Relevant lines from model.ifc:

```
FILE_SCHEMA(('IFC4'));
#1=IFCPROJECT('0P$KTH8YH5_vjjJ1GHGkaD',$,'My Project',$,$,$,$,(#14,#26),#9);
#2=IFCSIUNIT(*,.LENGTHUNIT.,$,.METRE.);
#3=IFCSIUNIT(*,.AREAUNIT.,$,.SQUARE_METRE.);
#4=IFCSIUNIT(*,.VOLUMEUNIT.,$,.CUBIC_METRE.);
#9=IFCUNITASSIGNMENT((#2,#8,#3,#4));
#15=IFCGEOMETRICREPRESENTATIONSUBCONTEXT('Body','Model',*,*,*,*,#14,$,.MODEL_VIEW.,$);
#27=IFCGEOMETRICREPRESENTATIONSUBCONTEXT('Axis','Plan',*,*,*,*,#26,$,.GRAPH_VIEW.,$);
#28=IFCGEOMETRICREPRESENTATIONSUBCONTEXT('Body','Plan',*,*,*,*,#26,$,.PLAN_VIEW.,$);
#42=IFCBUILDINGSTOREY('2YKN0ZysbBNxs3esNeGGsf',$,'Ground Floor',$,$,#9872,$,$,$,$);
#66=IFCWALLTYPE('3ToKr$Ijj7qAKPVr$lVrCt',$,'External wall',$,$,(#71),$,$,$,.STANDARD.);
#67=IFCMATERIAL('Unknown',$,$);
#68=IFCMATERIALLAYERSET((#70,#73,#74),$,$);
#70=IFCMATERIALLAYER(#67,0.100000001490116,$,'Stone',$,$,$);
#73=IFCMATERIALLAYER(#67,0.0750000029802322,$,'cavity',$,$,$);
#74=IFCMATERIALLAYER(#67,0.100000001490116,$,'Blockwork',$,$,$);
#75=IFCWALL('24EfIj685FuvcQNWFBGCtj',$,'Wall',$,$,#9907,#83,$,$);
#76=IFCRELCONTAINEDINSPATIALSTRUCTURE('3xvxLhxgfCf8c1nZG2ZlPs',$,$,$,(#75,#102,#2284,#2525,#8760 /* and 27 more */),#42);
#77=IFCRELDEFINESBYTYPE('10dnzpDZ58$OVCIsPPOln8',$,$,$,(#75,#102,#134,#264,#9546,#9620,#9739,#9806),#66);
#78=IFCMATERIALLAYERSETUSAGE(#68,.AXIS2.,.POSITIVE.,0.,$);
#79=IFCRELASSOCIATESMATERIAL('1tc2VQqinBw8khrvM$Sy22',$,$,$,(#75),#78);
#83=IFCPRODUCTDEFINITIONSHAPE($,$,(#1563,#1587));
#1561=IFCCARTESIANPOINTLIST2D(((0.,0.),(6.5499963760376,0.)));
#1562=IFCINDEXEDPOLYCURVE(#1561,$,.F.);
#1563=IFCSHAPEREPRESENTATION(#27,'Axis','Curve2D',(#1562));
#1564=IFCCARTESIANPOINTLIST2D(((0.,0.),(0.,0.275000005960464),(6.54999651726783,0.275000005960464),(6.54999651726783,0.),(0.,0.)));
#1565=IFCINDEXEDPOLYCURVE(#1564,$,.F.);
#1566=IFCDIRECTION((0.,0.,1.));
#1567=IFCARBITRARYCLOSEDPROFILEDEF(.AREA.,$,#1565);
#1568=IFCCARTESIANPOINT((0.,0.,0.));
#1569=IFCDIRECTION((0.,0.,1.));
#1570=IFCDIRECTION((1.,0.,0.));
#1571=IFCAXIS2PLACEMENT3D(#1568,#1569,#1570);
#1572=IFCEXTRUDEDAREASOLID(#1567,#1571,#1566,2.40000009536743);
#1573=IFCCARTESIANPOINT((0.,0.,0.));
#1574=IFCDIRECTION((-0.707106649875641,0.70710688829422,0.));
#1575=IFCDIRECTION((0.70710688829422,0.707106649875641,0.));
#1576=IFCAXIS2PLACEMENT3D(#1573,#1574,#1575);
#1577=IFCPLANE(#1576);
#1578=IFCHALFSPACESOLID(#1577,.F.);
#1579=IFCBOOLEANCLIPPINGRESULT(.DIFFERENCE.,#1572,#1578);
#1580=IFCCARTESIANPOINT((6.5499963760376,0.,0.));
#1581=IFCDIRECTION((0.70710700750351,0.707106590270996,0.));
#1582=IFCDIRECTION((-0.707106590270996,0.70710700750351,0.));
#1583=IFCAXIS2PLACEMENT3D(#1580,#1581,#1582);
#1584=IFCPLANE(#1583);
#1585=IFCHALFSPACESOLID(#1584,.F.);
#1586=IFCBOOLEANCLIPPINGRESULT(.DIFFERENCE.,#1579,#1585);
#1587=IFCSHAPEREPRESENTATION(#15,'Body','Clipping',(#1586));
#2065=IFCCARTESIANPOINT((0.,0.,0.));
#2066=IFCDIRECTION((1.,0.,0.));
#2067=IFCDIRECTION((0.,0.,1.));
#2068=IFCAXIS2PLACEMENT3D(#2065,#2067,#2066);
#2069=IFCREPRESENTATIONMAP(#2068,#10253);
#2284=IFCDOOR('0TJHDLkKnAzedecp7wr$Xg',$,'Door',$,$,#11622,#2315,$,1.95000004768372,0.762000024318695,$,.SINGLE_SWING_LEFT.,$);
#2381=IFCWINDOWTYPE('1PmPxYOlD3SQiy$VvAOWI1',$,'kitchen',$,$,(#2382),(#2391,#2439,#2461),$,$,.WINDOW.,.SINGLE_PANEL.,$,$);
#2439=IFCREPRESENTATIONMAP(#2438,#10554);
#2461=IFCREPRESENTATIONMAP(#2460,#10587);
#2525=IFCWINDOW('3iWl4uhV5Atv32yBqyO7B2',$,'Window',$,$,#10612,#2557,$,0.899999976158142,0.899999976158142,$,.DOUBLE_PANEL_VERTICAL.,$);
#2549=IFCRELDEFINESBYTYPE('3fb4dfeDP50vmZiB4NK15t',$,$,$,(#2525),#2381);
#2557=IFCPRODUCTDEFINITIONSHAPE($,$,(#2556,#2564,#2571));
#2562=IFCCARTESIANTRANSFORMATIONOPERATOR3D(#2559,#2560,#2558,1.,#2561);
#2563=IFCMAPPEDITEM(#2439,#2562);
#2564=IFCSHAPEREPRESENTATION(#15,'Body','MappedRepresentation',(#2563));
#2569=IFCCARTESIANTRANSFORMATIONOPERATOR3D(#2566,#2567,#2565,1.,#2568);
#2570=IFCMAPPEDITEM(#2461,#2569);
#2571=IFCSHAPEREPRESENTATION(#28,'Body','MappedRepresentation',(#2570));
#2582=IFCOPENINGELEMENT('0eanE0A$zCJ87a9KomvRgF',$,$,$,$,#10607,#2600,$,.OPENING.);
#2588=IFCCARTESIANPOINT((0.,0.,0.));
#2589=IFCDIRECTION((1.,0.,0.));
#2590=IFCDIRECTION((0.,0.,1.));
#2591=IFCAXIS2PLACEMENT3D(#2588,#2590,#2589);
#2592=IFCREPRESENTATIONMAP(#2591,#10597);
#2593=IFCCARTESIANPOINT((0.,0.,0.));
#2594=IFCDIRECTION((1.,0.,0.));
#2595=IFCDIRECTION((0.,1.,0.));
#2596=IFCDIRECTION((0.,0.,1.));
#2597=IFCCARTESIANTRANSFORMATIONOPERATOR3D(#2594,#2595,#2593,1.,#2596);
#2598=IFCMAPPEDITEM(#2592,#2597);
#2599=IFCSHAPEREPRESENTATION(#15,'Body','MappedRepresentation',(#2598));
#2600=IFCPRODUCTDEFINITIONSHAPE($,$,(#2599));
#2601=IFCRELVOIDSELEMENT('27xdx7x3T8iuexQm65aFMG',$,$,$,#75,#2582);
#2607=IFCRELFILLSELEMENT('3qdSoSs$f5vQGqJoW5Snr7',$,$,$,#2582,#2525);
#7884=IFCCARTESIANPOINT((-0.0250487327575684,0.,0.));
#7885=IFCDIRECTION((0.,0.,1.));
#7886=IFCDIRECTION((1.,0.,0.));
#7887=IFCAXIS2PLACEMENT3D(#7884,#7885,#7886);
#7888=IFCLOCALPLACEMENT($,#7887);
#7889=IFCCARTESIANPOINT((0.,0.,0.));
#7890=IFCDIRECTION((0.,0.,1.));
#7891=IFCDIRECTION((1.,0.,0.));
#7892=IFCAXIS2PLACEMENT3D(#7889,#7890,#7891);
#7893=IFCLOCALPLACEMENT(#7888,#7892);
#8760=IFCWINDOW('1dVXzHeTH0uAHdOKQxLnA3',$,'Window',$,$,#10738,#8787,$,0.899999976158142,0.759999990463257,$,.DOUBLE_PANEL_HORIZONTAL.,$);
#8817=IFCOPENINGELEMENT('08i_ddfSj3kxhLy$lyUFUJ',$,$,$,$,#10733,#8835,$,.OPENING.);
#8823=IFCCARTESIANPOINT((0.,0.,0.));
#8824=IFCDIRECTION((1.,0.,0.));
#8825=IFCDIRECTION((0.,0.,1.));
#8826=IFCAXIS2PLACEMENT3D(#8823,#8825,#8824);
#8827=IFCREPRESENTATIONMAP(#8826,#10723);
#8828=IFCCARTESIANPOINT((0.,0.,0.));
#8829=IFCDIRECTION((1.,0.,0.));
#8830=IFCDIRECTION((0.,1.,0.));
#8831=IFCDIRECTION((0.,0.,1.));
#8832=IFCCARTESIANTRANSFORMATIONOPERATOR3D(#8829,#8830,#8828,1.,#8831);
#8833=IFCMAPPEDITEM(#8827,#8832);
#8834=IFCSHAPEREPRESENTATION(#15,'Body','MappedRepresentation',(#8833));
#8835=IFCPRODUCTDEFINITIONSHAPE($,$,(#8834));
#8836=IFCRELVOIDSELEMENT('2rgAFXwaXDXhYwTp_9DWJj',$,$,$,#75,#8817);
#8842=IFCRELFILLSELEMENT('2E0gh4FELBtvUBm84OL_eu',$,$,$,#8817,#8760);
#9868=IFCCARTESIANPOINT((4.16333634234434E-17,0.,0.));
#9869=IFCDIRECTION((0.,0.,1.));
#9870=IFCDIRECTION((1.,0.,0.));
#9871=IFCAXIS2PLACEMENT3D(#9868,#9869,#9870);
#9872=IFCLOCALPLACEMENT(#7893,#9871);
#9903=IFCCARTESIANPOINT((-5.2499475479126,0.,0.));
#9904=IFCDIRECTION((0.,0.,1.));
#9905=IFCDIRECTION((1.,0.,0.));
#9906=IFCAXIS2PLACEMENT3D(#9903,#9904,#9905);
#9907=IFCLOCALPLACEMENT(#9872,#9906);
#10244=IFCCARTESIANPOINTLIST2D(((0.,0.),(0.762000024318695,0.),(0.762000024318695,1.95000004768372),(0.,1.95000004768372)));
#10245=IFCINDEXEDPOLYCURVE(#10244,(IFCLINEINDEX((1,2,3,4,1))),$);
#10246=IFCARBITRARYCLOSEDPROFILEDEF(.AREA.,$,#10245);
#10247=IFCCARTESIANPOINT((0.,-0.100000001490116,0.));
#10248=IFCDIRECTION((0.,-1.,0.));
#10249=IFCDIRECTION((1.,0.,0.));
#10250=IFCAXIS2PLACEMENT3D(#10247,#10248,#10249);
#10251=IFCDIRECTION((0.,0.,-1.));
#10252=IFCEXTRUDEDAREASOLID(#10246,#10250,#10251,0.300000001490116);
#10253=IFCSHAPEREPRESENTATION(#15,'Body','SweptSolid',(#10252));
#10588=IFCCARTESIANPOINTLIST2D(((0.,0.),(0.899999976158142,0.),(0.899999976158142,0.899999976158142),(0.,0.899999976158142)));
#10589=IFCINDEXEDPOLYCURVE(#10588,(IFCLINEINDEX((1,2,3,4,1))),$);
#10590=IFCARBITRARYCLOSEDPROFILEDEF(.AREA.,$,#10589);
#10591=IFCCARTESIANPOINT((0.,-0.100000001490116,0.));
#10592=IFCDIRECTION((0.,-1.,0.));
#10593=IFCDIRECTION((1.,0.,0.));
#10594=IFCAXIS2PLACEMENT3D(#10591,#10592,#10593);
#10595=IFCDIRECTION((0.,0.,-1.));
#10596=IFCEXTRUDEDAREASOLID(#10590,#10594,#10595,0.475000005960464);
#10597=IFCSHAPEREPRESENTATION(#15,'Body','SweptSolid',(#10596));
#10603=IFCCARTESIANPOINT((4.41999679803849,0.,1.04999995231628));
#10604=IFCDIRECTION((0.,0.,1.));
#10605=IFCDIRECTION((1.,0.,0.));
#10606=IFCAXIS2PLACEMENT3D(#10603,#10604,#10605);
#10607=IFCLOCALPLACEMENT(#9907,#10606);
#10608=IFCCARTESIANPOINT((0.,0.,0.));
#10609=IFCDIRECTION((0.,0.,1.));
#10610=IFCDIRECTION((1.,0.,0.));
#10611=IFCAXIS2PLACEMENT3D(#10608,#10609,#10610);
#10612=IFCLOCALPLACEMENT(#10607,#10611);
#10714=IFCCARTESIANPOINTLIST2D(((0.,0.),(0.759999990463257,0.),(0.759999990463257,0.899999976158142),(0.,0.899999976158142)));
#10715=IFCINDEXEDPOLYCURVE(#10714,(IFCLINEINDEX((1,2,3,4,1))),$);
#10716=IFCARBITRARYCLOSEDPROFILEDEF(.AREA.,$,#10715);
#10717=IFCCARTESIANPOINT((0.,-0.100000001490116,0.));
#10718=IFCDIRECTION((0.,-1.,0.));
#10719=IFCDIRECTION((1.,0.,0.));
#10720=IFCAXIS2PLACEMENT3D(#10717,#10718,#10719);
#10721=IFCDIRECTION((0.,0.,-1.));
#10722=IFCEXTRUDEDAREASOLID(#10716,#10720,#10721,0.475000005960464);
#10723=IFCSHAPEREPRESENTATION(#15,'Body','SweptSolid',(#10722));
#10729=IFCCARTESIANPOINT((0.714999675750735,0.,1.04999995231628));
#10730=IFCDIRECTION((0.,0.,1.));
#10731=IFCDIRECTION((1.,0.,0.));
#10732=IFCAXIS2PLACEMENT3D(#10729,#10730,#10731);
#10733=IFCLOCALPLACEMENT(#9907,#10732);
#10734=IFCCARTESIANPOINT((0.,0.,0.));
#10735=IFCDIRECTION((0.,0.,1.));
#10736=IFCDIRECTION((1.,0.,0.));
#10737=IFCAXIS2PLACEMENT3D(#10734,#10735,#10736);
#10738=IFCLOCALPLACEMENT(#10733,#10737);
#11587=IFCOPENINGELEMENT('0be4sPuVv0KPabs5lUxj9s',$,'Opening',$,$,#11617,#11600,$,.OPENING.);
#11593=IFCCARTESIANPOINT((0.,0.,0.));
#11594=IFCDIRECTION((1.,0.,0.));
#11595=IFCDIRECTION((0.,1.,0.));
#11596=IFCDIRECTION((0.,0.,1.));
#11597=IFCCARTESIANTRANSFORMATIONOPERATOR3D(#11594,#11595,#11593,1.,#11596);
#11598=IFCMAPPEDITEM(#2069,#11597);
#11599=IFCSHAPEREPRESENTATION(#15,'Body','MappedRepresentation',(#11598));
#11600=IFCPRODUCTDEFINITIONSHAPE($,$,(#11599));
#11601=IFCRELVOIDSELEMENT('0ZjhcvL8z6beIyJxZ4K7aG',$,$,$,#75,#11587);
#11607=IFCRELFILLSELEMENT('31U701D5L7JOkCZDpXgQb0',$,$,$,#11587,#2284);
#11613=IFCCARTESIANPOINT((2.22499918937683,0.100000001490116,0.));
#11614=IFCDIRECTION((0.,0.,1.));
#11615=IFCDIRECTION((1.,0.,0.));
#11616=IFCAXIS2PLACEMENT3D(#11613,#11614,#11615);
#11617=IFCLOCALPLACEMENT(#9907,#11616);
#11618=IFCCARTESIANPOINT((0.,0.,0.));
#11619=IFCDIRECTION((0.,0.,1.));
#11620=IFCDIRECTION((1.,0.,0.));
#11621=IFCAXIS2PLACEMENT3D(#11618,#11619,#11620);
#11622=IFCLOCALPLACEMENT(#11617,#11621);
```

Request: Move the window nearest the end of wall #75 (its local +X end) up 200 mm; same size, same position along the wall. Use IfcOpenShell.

```python
import numpy as np
import ifcopenshell
import ifcopenshell.api.geometry
import ifcopenshell.util.placement
import ifcopenshell.util.unit

model = ifcopenshell.open("model.ifc")
unit_scale = ifcopenshell.util.unit.calculate_unit_scale(model)

window = model.by_guid("3iWl4uhV5Atv32yBqyO7B2")
opening = window.FillsVoids[0].RelatingOpeningElement
dz = 0.2 / unit_scale

shift = np.array([0.0, 0.0, dz])
# The window is placed relative to its opening, so it follows when the opening moves.
matrix = ifcopenshell.util.placement.get_local_placement(opening.ObjectPlacement)
matrix[:3, 3] += shift
ifcopenshell.api.geometry.edit_object_placement(
    model, product=opening, matrix=matrix, is_si=False, should_transform_children=True
)

print(f"moved by {dz * unit_scale:+.3f} m")

model.write("model_edited.ifc")
```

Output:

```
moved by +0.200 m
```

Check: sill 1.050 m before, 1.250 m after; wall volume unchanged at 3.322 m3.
